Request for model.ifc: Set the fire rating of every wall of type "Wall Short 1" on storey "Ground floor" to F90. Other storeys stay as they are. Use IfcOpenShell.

First a look at what the model holds.

```python
import ifcopenshell
import ifcopenshell.util.element

model = ifcopenshell.open("model.ifc")
print(model.schema)
storey = next(s for s in model.by_type("IfcBuildingStorey") if s.Name == "Ground floor")
walls = [e for e in ifcopenshell.util.element.get_decomposition(storey) if e.is_a("IfcWall")]
seen = {}
for e in walls:
    element_type = ifcopenshell.util.element.get_type(e)
    key = (element_type.Name if element_type != e and element_type else None, ifcopenshell.util.element.get_pset(e, "Pset_WallCommon", "FireRating"))
    seen[key] = seen.get(key, 0) + 1
for (name, value), count in sorted(seen.items(), key=str):
    print(count, "x", name, "|", value)
```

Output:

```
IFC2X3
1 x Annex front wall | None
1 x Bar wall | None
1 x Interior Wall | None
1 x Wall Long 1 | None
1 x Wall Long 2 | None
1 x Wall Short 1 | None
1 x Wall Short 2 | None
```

```python
import ifcopenshell
import ifcopenshell.api.pset
import ifcopenshell.util.element

model = ifcopenshell.open("model.ifc")

storey = next(s for s in model.by_type("IfcBuildingStorey") if s.Name == "Ground floor")
walls = [e for e in ifcopenshell.util.element.get_decomposition(storey) if e.is_a("IfcWall")]

count = 0
for e in walls:
    element_type = ifcopenshell.util.element.get_type(e)
    if element_type in (None, e) or element_type.Name != "Wall Short 1":
        continue
    # add_pset returns the element's existing set when there is one.
    pset = ifcopenshell.api.pset.add_pset(model, product=e, name="Pset_WallCommon")
    ifcopenshell.api.pset.edit_pset(model, pset=pset, properties={"FireRating": "F90"})
    count += 1

print(count, "walls updated")

model.write("model_rev.ifc")
```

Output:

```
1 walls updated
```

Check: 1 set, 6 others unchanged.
